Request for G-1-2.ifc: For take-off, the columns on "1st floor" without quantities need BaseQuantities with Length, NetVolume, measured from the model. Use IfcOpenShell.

First a look at what the model holds.

```python
import ifcopenshell
import ifcopenshell.util.element
import ifcopenshell.util.unit

model = ifcopenshell.open("G-1-2.ifc")
print(model.schema)
for unit_type in ("LENGTHUNIT", "AREAUNIT", "VOLUMEUNIT"):
    print(unit_type, ifcopenshell.util.unit.calculate_unit_scale(model, unit_type))
storey = next(s for s in model.by_type("IfcBuildingStorey") if s.Name == "1st floor")
columns = [e for e in ifcopenshell.util.element.get_decomposition(storey) if e.is_a("IfcColumn")]
for e in sorted(columns, key=lambda e: e.id()):
    print(e.id(), e.is_a(), e.Name, list(ifcopenshell.util.element.get_psets(e, qtos_only=True)), sep=" | ")
```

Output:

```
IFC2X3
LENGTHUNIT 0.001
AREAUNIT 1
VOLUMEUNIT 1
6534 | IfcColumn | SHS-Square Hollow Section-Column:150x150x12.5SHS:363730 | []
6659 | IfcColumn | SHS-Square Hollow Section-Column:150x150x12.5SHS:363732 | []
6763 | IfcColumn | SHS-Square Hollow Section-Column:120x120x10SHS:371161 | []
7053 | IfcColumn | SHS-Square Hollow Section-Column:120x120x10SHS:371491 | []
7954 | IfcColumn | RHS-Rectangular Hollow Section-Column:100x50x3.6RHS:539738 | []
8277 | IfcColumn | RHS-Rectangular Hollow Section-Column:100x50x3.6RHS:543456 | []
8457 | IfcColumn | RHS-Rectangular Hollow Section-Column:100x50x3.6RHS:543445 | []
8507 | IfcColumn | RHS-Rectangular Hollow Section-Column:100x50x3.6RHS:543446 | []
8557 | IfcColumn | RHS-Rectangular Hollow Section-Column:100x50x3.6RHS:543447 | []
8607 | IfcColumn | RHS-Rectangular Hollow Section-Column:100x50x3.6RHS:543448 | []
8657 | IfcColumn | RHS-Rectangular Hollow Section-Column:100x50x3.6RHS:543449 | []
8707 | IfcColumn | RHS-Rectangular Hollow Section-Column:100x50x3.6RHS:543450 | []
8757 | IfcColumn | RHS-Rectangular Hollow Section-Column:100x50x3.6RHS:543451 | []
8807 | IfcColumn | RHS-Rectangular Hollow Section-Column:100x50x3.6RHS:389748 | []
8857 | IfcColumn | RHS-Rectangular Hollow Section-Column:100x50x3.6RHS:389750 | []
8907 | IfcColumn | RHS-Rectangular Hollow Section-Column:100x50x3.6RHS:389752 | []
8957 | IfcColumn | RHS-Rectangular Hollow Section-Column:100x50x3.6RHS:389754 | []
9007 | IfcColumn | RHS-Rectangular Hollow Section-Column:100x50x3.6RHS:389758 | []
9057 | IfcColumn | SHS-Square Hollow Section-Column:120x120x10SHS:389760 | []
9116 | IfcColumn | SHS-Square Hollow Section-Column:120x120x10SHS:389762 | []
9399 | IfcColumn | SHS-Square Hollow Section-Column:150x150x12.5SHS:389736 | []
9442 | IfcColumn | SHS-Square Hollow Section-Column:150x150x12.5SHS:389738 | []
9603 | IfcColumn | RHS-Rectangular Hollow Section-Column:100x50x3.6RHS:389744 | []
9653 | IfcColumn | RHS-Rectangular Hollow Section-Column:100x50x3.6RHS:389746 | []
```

```python
import ifcopenshell
import ifcopenshell.api.pset
import ifcopenshell.geom
import ifcopenshell.util.element
import ifcopenshell.util.shape
import ifcopenshell.util.unit

model = ifcopenshell.open("G-1-2.ifc")
unit_scale = ifcopenshell.util.unit.calculate_unit_scale(model)
volume_scale = ifcopenshell.util.unit.calculate_unit_scale(model, "VOLUMEUNIT")
settings = ifcopenshell.geom.settings()

storey = next(s for s in model.by_type("IfcBuildingStorey") if s.Name == "1st floor")
columns = [e for e in ifcopenshell.util.element.get_decomposition(storey) if e.is_a("IfcColumn")]

for e in sorted(columns, key=lambda e: e.id()):
    if ifcopenshell.util.element.get_psets(e, qtos_only=True, should_inherit=False):
        continue
    # Geometry comes back in metres, in the element's own axes.
    shape = ifcopenshell.geom.create_shape(settings, e)
    values = {
        "Length": ifcopenshell.util.shape.get_z(shape.geometry) / unit_scale,
        "NetVolume": ifcopenshell.util.shape.get_volume(shape.geometry) / volume_scale,
    }
    qto = ifcopenshell.api.pset.add_qto(model, product=e, name="BaseQuantities")
    ifcopenshell.api.pset.edit_qto(model, qto=qto, properties=values)
    print(e.id(), {k: round(v, 3) for k, v in values.items()})

model.write("G-1-2_updated.ifc")
```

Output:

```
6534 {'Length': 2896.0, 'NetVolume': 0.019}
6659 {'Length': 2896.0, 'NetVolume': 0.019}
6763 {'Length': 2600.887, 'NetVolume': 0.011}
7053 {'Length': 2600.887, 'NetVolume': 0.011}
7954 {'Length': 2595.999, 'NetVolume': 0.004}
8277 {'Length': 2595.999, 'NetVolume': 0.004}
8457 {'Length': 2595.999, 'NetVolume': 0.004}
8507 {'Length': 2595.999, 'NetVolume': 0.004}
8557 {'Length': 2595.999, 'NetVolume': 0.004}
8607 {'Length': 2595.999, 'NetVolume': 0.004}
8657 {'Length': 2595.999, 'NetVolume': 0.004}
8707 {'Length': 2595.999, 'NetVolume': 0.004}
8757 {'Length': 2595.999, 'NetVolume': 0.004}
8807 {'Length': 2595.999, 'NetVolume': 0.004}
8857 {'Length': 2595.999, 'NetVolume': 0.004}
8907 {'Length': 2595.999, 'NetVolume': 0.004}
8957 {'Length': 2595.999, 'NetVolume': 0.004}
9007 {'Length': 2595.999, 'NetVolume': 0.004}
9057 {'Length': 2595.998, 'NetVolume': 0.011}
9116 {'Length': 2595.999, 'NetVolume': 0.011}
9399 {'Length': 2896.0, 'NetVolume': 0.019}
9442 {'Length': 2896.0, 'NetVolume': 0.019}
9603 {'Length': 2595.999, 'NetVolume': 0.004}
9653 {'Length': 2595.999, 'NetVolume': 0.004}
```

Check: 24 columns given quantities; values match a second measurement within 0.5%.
